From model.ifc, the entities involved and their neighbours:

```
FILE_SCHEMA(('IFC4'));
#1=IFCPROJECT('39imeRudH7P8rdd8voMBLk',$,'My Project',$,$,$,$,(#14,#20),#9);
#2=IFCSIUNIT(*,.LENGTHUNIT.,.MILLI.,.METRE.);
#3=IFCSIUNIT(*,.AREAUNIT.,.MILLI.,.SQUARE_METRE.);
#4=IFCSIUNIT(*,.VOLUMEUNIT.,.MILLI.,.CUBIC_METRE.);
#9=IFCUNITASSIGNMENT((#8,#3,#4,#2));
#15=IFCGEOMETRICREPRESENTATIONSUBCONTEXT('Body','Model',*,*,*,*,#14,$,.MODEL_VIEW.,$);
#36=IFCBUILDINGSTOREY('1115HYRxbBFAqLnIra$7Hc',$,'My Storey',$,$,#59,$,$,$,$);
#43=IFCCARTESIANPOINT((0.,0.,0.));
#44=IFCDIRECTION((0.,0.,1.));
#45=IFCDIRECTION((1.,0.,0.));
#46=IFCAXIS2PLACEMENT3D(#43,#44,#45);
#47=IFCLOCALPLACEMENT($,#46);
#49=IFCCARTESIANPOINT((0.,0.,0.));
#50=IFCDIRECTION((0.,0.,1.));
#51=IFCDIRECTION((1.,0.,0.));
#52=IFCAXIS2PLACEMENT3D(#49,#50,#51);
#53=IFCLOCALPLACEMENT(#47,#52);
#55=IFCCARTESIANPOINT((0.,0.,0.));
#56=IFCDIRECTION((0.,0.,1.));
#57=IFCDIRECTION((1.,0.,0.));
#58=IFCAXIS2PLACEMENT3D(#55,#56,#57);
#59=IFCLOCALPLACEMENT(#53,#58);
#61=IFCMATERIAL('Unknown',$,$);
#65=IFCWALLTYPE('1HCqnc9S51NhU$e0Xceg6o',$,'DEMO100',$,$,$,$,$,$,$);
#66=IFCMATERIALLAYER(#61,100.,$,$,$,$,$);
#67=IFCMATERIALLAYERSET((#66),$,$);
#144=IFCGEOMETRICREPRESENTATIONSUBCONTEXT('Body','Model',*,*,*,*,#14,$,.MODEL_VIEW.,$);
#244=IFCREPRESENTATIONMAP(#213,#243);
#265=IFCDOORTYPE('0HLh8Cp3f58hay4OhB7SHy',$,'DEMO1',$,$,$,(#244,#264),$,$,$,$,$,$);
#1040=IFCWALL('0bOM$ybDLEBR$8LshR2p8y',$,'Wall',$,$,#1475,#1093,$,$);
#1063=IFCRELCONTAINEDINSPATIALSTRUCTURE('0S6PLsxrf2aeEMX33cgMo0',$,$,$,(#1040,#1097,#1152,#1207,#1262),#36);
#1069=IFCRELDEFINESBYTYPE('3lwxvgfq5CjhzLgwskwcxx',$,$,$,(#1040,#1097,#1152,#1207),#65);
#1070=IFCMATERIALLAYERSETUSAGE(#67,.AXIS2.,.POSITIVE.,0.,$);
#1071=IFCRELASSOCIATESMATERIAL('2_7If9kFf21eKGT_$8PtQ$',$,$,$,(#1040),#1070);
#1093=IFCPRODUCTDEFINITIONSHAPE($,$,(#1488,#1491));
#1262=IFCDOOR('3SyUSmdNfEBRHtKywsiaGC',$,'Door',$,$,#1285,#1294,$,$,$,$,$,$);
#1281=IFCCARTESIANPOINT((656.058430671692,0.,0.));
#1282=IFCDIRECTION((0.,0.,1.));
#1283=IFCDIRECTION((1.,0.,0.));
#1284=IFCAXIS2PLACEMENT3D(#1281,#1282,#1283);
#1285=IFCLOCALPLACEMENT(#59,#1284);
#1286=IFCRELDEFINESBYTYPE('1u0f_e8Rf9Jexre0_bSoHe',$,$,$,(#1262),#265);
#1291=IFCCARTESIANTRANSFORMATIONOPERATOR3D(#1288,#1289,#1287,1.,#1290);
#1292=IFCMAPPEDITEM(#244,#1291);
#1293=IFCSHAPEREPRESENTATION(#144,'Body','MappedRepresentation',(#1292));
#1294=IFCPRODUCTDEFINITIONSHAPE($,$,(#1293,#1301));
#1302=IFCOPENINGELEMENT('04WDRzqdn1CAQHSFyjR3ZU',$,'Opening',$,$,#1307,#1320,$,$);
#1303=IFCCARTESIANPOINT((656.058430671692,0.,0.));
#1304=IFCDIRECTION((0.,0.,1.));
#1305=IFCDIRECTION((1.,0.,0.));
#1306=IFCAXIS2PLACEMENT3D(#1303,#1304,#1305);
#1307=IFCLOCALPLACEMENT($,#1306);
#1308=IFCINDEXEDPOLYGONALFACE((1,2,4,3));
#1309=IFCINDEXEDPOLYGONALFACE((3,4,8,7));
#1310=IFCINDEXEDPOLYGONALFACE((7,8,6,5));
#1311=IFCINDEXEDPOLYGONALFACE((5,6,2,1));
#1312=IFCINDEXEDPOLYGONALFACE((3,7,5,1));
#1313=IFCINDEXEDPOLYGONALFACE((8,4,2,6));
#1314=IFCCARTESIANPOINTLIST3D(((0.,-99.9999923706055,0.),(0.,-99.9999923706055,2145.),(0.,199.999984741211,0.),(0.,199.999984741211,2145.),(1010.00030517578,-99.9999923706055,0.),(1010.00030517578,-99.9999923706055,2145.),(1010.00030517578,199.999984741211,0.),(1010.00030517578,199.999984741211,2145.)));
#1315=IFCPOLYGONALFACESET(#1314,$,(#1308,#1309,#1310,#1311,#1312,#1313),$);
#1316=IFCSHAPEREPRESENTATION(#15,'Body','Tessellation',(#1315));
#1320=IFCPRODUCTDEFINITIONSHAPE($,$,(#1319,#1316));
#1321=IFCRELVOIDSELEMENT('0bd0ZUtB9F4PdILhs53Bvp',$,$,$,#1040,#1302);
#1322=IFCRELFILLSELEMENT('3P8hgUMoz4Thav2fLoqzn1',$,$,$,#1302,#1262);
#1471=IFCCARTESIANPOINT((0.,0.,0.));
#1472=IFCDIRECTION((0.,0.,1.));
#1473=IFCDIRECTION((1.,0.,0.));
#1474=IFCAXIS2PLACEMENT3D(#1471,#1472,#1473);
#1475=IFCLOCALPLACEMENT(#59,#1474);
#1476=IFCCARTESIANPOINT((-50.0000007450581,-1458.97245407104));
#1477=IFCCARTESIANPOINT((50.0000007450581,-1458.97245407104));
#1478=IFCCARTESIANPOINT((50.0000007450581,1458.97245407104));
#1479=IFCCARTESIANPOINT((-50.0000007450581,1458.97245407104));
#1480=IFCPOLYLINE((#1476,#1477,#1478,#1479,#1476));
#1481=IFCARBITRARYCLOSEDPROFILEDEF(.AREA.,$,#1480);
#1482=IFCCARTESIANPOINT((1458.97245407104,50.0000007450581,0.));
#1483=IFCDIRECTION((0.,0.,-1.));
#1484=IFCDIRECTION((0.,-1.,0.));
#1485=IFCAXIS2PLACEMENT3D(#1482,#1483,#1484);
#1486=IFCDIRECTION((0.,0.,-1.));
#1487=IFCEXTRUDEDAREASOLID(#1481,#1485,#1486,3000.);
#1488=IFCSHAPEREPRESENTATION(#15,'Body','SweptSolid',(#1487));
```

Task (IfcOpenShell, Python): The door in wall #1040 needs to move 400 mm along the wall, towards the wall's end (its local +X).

```python
import ifcopenshell
import ifcopenshell.api.geometry
import ifcopenshell.util.placement

model = ifcopenshell.open("model.ifc")

door = model.by_guid("3SyUSmdNfEBRHtKywsiaGC")
opening = door.FillsVoids[0].RelatingOpeningElement
wall = opening.VoidsElements[0].RelatingBuildingElement

wall_matrix = ifcopenshell.util.placement.get_local_placement(wall.ObjectPlacement)
shift = wall_matrix[:3, 0] * 400.0
before = ifcopenshell.util.placement.get_local_placement(door.ObjectPlacement)[:3, 3].copy()

# The door is not placed relative to its opening, so move both.
for product in (opening, door):
    matrix = ifcopenshell.util.placement.get_local_placement(product.ObjectPlacement)
    matrix[:3, 3] += shift
    ifcopenshell.api.geometry.edit_object_placement(model, product=product, matrix=matrix, is_si=False)

after = ifcopenshell.util.placement.get_local_placement(door.ObjectPlacement)[:3, 3]
print("door moved by", (after - before).round(3) + 0.0)

model.write("model_v2.ifc")
```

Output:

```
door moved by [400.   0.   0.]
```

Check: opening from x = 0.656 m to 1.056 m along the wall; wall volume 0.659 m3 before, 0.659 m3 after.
